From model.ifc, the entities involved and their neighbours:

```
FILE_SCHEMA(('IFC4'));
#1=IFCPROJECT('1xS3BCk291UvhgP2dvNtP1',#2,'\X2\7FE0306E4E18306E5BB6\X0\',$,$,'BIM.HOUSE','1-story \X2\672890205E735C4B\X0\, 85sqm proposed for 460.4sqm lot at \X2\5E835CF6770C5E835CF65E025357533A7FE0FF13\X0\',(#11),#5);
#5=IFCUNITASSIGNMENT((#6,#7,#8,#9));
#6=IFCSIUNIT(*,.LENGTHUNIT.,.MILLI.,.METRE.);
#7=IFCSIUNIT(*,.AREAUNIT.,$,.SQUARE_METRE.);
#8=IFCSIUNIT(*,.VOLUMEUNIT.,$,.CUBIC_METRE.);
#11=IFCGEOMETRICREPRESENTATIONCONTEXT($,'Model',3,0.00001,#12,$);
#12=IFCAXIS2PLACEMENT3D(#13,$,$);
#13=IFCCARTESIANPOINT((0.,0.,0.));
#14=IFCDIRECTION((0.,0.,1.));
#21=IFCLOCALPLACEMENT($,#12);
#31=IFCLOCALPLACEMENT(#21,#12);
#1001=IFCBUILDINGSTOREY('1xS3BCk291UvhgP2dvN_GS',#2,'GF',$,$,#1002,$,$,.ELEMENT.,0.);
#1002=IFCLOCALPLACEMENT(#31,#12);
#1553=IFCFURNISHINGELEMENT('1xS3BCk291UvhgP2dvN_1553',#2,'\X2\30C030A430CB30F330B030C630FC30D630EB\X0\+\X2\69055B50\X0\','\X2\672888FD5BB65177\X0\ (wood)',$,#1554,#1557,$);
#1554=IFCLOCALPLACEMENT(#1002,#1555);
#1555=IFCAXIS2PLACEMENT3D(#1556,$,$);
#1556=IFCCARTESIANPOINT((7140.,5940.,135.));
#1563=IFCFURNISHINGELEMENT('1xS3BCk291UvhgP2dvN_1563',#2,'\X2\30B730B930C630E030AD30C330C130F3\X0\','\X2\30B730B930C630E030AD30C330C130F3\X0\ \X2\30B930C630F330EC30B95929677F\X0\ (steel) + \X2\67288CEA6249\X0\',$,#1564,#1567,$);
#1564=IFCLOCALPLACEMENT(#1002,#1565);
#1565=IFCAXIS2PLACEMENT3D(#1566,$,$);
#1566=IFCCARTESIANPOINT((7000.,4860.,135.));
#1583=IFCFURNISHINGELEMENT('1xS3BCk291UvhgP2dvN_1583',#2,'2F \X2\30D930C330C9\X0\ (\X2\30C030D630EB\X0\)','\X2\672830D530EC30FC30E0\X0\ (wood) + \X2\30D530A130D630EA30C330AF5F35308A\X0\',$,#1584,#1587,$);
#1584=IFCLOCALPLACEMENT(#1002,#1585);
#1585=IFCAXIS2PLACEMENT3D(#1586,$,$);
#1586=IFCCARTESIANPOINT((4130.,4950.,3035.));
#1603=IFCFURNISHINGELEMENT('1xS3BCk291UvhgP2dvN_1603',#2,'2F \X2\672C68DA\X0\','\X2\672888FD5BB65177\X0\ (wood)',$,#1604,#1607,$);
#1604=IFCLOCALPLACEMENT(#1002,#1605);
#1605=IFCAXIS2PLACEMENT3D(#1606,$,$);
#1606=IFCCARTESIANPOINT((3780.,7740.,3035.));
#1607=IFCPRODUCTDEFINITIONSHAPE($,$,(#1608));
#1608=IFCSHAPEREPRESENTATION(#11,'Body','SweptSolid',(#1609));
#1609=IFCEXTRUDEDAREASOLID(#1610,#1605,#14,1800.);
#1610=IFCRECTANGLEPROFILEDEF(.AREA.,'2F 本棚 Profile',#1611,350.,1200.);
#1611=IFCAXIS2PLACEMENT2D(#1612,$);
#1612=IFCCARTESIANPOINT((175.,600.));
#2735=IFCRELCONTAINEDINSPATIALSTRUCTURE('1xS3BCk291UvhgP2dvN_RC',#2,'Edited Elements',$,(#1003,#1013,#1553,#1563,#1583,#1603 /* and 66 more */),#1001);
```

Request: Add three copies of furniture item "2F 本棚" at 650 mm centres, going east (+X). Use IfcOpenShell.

```python
import numpy as np
import ifcopenshell
import ifcopenshell.api.geometry
import ifcopenshell.api.root
import ifcopenshell.util.element
import ifcopenshell.util.placement
import ifcopenshell.util.unit

model = ifcopenshell.open("model.ifc")
unit_scale = ifcopenshell.util.unit.calculate_unit_scale(model)


def reuse_history(source, copy):
    """copy_class also copies each property set's owner history, people and application; keep the originals."""
    for rel in copy.IsDefinedBy:
        if rel.is_a("IfcRelDefinesByProperties") and (history := rel.RelatingPropertyDefinition.OwnerHistory):
            rel.RelatingPropertyDefinition.OwnerHistory = source.OwnerHistory
            ifcopenshell.util.element.remove_deep2(model, history)


source = model.by_guid("1xS3BCk291UvhgP2dvN_1603")
base = ifcopenshell.util.placement.get_local_placement(source.ObjectPlacement)
step = np.array([1.0, 0.0, 0.0]) * 0.65 / unit_scale

for i in range(1, 4):
    copy = ifcopenshell.api.root.copy_class(model, product=source)
    copy.Representation = ifcopenshell.util.element.copy_deep(
        model, source.Representation, exclude=["IfcGeometricRepresentationContext", "IfcRepresentationMap"]
    )
    reuse_history(source, copy)
    matrix = base.copy()
    matrix[:3, 3] += i * step
    print("added at", matrix[:3, 3].round(3) + 0.0)
    ifcopenshell.api.geometry.edit_object_placement(model, product=copy, matrix=matrix, is_si=False)

model.write("model_edited.ifc")
```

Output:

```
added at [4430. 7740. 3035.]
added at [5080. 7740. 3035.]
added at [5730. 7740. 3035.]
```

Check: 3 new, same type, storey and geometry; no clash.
